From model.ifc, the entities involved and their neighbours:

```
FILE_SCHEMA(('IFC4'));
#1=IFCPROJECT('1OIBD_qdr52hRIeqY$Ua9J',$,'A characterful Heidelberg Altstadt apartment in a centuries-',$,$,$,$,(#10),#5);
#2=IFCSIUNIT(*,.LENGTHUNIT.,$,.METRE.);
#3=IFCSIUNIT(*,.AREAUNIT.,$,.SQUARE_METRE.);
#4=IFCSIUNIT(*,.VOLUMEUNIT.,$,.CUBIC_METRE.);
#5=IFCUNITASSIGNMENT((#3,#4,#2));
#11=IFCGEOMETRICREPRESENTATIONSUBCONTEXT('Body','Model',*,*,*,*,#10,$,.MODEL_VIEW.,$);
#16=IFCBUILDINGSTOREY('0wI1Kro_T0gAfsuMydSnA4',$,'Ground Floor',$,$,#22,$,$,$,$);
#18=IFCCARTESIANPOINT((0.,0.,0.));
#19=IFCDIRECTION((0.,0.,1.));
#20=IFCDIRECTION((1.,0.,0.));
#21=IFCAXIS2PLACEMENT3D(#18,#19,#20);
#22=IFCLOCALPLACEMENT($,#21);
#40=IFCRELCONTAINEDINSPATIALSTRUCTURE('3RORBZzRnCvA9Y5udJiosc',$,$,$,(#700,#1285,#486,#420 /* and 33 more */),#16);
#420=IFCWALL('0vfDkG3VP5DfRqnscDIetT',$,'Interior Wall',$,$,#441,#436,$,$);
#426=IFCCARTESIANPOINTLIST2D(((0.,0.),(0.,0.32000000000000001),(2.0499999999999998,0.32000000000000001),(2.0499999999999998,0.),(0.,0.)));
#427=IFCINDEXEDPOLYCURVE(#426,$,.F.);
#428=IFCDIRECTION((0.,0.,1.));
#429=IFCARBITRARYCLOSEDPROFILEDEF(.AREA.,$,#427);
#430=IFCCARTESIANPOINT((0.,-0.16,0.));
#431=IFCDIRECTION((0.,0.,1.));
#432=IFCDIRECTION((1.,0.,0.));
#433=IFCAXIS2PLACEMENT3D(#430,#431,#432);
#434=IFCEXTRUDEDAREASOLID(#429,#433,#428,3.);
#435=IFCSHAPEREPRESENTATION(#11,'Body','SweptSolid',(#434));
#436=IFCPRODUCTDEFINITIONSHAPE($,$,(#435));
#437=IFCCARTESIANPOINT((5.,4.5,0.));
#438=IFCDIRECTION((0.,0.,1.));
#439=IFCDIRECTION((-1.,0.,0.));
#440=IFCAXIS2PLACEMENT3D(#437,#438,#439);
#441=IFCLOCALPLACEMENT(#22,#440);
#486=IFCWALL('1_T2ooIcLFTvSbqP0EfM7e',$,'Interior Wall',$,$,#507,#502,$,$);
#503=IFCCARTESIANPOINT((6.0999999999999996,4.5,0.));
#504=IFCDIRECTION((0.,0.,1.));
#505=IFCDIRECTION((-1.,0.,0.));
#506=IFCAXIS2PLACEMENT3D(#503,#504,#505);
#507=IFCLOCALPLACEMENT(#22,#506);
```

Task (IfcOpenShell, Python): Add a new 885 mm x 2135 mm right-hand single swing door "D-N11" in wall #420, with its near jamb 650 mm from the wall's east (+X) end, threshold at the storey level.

```python
import numpy as np
import ifcopenshell
import ifcopenshell.api.feature
import ifcopenshell.api.geometry
import ifcopenshell.api.root
import ifcopenshell.api.spatial
import ifcopenshell.geom
import ifcopenshell.util.element
import ifcopenshell.util.placement
import ifcopenshell.util.representation
import ifcopenshell.util.shape
import ifcopenshell.util.unit

model = ifcopenshell.open("model.ifc")
unit_scale = ifcopenshell.util.unit.calculate_unit_scale(model)
settings = ifcopenshell.geom.settings()


def volume(element):
    """Net volume in cubic metres, openings subtracted."""
    shape = ifcopenshell.geom.create_shape(settings, element)
    return ifcopenshell.util.shape.get_volume(shape.geometry)


wall = model.by_guid("0vfDkG3VP5DfRqnscDIetT")
storey = ifcopenshell.util.element.get_container(wall, ifc_class="IfcBuildingStorey")
context = ifcopenshell.util.representation.get_context(model, "Model", "Body", "MODEL_VIEW")
before = volume(wall)

width, height, from_end, sill = 0.885, 2.135, 0.65, 0.0  # metres

# The wall runs along its own X axis, and the end named is its -X end.
wall_shape = ifcopenshell.geom.create_shape(settings, wall)
x, y, z = ifcopenshell.util.shape.get_vertices(wall_shape.geometry).T
start = x.min() + from_end
face, thickness = float(y.min()), float(y.max() - y.min())
wall_matrix = ifcopenshell.util.placement.get_local_placement(wall.ObjectPlacement)
level = ifcopenshell.util.placement.get_local_placement(storey.ObjectPlacement)[2, 3]


def in_wall(x, y):
    """Placement at x, y metres in the wall's axes, at sill height."""
    matrix = wall_matrix.copy()
    matrix[:, 3] = wall_matrix @ np.array([x / unit_scale, y / unit_scale, 0.0, 1.0])
    matrix[2, 3] = level + sill / unit_scale
    return matrix


# Opening: a box that overshoots both wall faces by 50 mm.
opening = ifcopenshell.api.root.create_entity(model, ifc_class="IfcOpeningElement", predefined_type="OPENING")
box = ifcopenshell.api.geometry.add_wall_representation(
    model, context=context, length=width, height=height, thickness=thickness + 0.1
)
ifcopenshell.api.geometry.assign_representation(model, product=opening, representation=box)
ifcopenshell.api.geometry.edit_object_placement(model, product=opening, matrix=in_wall(start, face - 0.05), is_si=False)
ifcopenshell.api.feature.add_feature(model, feature=opening, element=wall)

door = ifcopenshell.api.root.create_entity(model, ifc_class="IfcDoor", name="D-N11", predefined_type="DOOR")
door.OverallWidth, door.OverallHeight = width / unit_scale, height / unit_scale
door.OperationType = "SINGLE_SWING_RIGHT"
body = ifcopenshell.api.geometry.add_door_representation(
    model,
    context=context,
    overall_width=door.OverallWidth,
    overall_height=door.OverallHeight,
    operation_type="SINGLE_SWING_RIGHT",
    lining_properties={"LiningDepth": thickness / unit_scale, "ThresholdDepth": thickness / unit_scale},
)
ifcopenshell.api.geometry.assign_representation(model, product=door, representation=body)
ifcopenshell.api.spatial.assign_container(model, products=[door], relating_structure=storey)
ifcopenshell.api.feature.add_filling(model, opening=opening, element=door)

# The lining spans the wall, so the door starts at the wall face.
ifcopenshell.api.geometry.edit_object_placement(model, product=door, matrix=in_wall(start, face), is_si=False)

after = volume(wall)

print(f"wall volume {before:.3f} -> {after:.3f} m3")

model.write("model_v2.ifc")
```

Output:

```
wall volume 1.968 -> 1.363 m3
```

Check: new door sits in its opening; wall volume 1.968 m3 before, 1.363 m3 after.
